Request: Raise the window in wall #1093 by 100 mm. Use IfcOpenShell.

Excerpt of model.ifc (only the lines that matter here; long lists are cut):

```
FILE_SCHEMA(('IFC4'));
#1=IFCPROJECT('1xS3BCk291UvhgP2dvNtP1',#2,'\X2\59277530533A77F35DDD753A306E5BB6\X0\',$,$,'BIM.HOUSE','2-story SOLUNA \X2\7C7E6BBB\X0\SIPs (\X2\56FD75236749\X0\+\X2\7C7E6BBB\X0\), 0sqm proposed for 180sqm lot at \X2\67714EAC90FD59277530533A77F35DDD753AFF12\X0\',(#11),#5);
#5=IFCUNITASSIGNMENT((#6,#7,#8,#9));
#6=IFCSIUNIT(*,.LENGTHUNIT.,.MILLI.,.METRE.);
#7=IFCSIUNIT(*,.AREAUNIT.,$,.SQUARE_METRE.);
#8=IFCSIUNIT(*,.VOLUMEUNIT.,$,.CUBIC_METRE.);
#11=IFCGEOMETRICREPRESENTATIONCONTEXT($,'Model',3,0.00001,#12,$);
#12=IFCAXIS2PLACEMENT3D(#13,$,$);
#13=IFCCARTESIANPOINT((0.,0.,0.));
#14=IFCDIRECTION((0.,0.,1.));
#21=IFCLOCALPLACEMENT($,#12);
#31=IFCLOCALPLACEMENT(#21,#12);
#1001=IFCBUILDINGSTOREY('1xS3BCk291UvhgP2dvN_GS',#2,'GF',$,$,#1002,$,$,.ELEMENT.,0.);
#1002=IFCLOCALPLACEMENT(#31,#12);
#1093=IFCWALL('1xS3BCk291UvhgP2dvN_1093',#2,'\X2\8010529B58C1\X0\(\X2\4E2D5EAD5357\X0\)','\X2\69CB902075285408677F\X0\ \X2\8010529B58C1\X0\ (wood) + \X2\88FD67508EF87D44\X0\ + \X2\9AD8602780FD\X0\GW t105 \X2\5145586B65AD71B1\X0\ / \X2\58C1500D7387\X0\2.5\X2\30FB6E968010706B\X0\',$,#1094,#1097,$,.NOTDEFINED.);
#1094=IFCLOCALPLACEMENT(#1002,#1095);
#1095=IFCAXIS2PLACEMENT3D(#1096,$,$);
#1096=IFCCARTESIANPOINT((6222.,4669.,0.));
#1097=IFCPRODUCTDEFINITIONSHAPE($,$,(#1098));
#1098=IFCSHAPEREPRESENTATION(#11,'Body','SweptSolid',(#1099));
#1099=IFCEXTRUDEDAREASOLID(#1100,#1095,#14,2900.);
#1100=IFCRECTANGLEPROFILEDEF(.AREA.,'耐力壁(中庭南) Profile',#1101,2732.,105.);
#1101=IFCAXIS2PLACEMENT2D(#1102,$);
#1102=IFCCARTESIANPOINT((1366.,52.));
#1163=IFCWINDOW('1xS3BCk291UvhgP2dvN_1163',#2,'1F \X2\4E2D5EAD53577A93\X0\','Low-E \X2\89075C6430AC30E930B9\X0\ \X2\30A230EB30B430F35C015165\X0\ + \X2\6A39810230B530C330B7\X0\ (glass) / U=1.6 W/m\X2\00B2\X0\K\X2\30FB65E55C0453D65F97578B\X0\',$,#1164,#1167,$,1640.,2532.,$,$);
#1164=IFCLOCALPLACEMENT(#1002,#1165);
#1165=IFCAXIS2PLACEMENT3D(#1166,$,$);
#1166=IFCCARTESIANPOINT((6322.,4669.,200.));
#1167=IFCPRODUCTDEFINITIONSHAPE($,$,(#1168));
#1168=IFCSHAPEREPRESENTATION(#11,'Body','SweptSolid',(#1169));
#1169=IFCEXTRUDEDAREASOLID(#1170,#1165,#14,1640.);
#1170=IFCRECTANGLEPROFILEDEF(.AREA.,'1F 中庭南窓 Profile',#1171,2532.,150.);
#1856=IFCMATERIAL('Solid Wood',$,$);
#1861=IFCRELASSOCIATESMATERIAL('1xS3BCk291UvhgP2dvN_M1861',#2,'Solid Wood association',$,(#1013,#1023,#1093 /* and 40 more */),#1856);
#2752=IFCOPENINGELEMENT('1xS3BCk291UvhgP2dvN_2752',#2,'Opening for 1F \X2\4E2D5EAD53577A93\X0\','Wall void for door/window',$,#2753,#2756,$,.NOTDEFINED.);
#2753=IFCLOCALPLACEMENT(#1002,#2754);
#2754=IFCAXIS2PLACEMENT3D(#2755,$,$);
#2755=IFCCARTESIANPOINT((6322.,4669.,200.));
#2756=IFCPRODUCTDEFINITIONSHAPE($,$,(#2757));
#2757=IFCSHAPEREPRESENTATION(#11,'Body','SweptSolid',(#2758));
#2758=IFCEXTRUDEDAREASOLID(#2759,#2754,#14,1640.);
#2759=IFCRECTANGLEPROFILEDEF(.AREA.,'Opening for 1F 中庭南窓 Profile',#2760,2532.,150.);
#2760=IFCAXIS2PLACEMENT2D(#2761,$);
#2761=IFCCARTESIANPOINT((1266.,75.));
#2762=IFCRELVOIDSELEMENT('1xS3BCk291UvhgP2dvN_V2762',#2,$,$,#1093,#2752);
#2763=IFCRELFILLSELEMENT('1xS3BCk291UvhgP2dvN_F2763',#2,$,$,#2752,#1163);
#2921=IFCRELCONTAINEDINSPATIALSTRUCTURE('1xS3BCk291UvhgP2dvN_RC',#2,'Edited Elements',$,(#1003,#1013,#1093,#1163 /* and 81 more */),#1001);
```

```python
import numpy as np
import ifcopenshell
import ifcopenshell.api.geometry
import ifcopenshell.util.placement
import ifcopenshell.util.unit

model = ifcopenshell.open("model.ifc")
unit_scale = ifcopenshell.util.unit.calculate_unit_scale(model)

window = model.by_guid("1xS3BCk291UvhgP2dvN_1163")
opening = window.FillsVoids[0].RelatingOpeningElement
dz = 100.0

shift = np.array([0.0, 0.0, dz])
# The window is not placed relative to its opening, so move both.
for product in (opening, window):
    matrix = ifcopenshell.util.placement.get_local_placement(product.ObjectPlacement)
    matrix[:3, 3] += shift
    ifcopenshell.api.geometry.edit_object_placement(model, product=product, matrix=matrix, is_si=False)

print(f"moved by {dz * unit_scale:+.3f} m")

model.write("model_edited.ifc")
```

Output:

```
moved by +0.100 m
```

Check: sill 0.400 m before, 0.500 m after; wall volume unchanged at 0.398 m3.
